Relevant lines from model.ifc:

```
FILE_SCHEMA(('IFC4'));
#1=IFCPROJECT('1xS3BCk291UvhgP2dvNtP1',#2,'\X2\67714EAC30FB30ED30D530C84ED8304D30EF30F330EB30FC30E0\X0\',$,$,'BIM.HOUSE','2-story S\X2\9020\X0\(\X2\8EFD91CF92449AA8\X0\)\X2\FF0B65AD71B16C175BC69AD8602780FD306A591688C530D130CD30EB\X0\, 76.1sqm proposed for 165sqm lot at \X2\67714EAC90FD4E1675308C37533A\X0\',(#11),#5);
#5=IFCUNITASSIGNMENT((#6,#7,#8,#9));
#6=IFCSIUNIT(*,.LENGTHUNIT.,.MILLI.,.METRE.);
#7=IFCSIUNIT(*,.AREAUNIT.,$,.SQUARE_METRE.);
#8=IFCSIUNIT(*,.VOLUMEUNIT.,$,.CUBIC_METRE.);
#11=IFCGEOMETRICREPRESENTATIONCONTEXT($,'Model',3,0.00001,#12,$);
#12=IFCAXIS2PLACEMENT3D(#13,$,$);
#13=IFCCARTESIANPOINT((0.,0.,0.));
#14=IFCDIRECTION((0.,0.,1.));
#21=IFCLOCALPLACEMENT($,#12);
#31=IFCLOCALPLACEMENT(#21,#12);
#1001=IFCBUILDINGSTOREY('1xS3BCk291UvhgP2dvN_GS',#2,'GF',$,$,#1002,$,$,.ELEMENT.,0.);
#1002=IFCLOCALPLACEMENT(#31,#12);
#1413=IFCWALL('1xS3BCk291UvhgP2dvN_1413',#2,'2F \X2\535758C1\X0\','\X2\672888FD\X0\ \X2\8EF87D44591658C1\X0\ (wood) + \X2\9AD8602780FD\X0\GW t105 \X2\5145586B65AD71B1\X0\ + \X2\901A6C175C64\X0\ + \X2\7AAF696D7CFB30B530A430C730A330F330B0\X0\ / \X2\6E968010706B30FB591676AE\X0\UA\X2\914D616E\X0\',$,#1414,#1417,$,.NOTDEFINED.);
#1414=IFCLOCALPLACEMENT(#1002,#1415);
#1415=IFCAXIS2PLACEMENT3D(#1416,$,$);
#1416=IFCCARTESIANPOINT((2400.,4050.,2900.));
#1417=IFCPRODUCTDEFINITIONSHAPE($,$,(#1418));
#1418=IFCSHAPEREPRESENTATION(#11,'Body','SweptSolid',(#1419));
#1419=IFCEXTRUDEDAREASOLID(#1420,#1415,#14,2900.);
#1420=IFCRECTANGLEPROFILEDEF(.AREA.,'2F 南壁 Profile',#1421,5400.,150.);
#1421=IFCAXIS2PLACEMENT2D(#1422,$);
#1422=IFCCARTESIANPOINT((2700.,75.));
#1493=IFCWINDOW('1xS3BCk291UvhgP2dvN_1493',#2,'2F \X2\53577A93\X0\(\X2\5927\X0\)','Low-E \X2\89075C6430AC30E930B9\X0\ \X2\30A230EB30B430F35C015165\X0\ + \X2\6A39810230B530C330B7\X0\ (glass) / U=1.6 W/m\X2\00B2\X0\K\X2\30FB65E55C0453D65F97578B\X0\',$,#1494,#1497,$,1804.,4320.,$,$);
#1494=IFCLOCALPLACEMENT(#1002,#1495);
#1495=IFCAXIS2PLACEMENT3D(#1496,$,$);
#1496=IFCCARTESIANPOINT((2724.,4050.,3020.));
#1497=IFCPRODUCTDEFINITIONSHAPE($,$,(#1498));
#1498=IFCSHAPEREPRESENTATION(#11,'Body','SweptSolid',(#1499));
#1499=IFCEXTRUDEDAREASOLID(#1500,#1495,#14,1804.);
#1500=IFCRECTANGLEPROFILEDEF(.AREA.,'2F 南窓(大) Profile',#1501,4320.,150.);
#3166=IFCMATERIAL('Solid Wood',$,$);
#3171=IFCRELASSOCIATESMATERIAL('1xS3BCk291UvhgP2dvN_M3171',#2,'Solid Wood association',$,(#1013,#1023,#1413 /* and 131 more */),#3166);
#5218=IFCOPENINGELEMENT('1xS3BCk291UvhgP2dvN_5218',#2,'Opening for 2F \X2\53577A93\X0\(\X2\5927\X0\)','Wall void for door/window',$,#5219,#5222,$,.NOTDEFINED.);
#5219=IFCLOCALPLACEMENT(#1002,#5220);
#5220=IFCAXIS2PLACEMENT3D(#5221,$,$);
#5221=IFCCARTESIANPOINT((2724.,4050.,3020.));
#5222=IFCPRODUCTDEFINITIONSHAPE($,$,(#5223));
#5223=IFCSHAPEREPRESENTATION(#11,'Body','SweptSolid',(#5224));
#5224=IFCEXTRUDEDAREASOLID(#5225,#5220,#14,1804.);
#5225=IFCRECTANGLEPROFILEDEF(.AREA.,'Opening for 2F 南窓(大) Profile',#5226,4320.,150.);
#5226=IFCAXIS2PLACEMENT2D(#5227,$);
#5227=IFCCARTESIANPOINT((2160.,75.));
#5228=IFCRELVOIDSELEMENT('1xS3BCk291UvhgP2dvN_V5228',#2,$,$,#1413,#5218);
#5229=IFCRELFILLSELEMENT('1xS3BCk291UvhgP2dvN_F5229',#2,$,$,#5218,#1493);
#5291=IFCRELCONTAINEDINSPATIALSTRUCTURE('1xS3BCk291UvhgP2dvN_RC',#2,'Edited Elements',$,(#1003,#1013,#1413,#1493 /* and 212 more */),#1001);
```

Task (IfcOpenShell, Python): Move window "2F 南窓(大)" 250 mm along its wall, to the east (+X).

```python
import ifcopenshell
import ifcopenshell.api.geometry
import ifcopenshell.util.placement
import ifcopenshell.util.unit

model = ifcopenshell.open("model.ifc")
unit_scale = ifcopenshell.util.unit.calculate_unit_scale(model)

window = model.by_id(1493)
opening = window.FillsVoids[0].RelatingOpeningElement
wall = opening.VoidsElements[0].RelatingBuildingElement

wall_matrix = ifcopenshell.util.placement.get_local_placement(wall.ObjectPlacement)
shift = wall_matrix[:3, 0] * 0.25 / unit_scale
before = ifcopenshell.util.placement.get_local_placement(window.ObjectPlacement)[:3, 3].copy()

# The window is not placed relative to its opening, so move both.
for product in (opening, window):
    matrix = ifcopenshell.util.placement.get_local_placement(product.ObjectPlacement)
    matrix[:3, 3] += shift
    ifcopenshell.api.geometry.edit_object_placement(model, product=product, matrix=matrix, is_si=False)

after = ifcopenshell.util.placement.get_local_placement(window.ObjectPlacement)[:3, 3]
print("window moved by", (after - before).round(3) + 0.0)

model.write("model_edited.ifc")
```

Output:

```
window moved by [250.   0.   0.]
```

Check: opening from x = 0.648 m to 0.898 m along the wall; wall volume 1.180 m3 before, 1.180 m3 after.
